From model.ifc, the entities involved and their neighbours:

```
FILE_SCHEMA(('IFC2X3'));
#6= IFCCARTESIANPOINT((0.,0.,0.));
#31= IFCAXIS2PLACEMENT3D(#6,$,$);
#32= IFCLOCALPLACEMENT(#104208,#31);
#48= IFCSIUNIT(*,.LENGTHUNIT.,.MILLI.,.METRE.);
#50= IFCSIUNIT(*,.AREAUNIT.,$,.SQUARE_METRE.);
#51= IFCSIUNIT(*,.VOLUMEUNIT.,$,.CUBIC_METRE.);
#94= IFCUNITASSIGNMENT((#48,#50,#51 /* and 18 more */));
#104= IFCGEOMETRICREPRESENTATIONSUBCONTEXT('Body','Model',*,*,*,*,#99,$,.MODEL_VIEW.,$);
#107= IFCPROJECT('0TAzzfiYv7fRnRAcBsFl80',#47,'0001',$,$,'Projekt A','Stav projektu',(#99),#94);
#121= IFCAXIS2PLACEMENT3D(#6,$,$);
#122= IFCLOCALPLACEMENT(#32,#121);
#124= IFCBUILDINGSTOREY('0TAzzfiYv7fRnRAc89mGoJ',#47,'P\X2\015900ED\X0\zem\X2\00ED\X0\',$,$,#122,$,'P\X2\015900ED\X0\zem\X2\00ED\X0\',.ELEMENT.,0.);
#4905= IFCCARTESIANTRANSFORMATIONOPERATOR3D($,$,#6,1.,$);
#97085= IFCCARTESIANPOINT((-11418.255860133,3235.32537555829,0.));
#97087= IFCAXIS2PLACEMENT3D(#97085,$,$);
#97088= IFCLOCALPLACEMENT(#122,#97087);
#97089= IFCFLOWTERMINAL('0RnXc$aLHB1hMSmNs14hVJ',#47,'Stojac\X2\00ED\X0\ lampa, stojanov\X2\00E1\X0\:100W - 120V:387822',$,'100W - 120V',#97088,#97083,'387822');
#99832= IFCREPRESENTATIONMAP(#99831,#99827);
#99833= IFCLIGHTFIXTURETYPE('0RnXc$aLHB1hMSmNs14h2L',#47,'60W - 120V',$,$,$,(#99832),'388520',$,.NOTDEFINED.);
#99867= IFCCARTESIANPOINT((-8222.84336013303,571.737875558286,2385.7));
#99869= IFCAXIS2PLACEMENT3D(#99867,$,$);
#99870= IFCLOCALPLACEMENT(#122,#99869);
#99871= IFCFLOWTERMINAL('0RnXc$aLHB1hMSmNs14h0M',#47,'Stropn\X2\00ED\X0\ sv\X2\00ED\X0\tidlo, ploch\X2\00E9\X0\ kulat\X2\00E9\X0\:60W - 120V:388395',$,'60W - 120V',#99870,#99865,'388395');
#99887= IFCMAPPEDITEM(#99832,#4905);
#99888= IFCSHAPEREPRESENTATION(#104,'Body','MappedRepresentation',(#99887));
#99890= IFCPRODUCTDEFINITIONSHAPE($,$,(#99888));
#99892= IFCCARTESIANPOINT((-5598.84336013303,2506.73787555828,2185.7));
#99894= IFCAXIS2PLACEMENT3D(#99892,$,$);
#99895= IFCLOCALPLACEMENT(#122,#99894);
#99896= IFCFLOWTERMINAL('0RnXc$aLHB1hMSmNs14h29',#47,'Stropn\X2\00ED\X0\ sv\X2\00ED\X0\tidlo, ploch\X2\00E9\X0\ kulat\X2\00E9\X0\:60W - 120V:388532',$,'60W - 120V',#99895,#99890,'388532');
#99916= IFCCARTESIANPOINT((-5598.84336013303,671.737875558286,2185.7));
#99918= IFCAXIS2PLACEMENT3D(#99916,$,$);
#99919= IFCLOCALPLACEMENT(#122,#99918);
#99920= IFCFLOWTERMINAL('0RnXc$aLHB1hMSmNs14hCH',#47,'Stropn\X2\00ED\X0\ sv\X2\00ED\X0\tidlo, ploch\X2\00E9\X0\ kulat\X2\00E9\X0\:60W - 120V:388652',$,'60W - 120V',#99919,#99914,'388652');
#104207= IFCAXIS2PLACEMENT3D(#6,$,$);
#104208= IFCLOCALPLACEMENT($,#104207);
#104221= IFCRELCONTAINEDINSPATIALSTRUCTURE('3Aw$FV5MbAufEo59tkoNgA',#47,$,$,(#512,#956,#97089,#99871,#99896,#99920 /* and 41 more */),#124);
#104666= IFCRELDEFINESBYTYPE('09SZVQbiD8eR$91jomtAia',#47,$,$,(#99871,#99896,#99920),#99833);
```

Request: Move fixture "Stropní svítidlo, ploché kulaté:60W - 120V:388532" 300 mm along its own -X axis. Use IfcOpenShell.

```python
import ifcopenshell
import ifcopenshell.api.geometry
import ifcopenshell.util.placement
import ifcopenshell.util.unit

model = ifcopenshell.open("model.ifc")
unit_scale = ifcopenshell.util.unit.calculate_unit_scale(model)

item = model.by_guid("0RnXc$aLHB1hMSmNs14h29")
matrix = ifcopenshell.util.placement.get_local_placement(item.ObjectPlacement)
matrix[:3, 3] -= matrix[:3, 0] * 0.3 / unit_scale
ifcopenshell.api.geometry.edit_object_placement(model, product=item, matrix=matrix, is_si=False)

print(ifcopenshell.util.placement.get_local_placement(item.ObjectPlacement).round(3) + 0.0)

model.write("model-out.ifc")
```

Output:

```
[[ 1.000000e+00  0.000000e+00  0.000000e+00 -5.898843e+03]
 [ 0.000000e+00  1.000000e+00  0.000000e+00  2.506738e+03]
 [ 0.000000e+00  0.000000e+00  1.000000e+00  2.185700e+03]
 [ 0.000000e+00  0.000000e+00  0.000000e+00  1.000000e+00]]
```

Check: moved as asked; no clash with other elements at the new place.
